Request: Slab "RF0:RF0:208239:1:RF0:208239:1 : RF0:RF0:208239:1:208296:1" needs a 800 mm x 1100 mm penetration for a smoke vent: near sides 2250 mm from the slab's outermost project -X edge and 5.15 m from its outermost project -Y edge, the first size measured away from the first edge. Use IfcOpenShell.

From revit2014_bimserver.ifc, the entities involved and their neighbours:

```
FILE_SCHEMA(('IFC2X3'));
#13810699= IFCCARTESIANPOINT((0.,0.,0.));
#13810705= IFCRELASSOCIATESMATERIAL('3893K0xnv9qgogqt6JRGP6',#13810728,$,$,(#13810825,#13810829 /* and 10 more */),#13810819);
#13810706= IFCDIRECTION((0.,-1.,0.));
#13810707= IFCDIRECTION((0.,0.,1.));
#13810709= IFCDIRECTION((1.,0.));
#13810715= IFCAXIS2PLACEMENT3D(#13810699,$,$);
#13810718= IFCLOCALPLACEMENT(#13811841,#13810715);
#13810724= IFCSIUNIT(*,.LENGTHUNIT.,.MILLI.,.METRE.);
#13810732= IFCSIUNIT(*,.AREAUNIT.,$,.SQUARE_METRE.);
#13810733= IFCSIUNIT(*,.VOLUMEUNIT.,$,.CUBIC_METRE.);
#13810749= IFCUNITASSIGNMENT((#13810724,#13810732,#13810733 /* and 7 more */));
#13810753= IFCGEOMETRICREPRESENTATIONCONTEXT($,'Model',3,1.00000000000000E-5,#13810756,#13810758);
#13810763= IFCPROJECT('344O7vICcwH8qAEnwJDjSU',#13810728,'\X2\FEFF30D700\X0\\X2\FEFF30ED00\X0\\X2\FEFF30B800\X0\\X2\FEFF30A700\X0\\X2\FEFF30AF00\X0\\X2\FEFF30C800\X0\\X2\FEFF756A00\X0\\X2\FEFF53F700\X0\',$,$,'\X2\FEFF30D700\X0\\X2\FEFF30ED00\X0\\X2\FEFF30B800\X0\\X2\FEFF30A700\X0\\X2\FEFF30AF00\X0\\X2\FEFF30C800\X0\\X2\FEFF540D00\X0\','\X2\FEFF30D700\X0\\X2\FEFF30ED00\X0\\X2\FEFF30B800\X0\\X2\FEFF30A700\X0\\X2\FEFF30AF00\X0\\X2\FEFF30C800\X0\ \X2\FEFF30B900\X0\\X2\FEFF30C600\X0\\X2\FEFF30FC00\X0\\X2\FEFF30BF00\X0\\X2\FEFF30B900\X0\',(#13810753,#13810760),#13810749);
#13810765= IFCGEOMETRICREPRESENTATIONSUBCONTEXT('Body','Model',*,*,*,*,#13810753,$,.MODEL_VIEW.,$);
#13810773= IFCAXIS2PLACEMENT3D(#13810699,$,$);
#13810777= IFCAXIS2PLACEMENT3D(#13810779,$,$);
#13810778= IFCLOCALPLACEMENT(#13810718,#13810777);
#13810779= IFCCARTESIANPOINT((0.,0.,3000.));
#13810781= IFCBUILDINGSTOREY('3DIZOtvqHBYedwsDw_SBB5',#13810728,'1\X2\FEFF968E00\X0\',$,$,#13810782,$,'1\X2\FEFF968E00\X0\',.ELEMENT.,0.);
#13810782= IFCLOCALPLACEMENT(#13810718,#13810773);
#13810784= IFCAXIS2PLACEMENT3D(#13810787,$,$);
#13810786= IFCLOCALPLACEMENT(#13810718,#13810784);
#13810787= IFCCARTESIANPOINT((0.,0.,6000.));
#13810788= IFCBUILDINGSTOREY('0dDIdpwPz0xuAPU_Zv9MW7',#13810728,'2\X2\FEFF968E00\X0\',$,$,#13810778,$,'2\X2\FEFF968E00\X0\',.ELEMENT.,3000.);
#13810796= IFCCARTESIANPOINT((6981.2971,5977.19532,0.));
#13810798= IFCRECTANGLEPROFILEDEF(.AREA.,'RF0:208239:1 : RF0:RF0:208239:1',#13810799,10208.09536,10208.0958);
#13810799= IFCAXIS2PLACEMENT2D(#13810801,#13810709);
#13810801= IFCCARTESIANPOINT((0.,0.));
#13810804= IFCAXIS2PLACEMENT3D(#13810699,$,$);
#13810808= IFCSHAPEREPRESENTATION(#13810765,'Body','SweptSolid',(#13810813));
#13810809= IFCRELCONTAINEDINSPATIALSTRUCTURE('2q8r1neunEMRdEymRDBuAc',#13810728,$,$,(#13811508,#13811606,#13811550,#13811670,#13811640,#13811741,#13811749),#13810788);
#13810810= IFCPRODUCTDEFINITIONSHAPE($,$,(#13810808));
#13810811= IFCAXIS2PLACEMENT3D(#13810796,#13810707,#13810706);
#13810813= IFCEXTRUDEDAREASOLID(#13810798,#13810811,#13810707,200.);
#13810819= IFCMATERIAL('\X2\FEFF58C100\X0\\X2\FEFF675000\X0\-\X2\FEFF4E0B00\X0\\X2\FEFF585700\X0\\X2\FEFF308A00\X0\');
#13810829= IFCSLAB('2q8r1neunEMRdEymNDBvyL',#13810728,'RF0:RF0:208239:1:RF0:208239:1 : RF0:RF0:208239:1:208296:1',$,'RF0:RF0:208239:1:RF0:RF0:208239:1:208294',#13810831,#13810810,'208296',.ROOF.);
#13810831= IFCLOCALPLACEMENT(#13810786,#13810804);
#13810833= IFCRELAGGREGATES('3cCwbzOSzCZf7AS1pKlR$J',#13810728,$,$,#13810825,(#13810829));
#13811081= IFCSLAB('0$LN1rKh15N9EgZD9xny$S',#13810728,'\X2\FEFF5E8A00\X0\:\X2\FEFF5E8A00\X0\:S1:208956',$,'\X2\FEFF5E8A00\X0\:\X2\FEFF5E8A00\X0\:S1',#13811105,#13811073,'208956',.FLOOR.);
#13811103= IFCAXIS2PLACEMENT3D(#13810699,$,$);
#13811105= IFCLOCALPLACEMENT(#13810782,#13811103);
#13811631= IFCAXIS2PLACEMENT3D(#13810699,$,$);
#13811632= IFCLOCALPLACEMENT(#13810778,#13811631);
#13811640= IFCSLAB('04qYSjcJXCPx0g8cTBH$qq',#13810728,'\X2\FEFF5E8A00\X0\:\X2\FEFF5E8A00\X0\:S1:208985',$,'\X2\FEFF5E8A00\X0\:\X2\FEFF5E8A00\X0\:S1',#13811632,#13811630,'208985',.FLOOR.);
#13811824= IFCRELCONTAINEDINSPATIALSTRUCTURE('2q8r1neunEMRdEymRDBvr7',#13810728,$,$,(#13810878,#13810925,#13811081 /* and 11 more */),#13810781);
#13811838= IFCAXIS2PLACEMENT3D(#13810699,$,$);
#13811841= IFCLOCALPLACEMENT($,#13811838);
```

```python
import numpy as np
import ifcopenshell
import ifcopenshell.api.feature
import ifcopenshell.api.geometry
import ifcopenshell.api.root
import ifcopenshell.geom
import ifcopenshell.util.placement
import ifcopenshell.util.representation
import ifcopenshell.util.shape
import ifcopenshell.util.unit

model = ifcopenshell.open("revit2014_bimserver.ifc")
unit_scale = ifcopenshell.util.unit.calculate_unit_scale(model)
settings = ifcopenshell.geom.settings()


def volume(element):
    """Net volume in cubic metres, openings subtracted."""
    shape = ifcopenshell.geom.create_shape(settings, element)
    return ifcopenshell.util.shape.get_volume(shape.geometry)


slab = model.by_id(13810829)
before = volume(slab)

# Extent in the slab's own axes, in metres. The edges named are its -X and -Y sides.
slab_shape = ifcopenshell.geom.create_shape(settings, slab)
vertices = ifcopenshell.util.shape.get_vertices(slab_shape.geometry)
x_min, y_min, bottom = vertices.min(axis=0)
top = vertices[:, 2].max()

opening = ifcopenshell.api.root.create_entity(model, ifc_class="IfcOpeningElement", name="Smoke vent opening")
context = ifcopenshell.util.representation.get_context(model, "Model", "Body", "MODEL_VIEW")
width, depth = 0.8, 1.1
outline = [(0.0, 0.0), (width, 0.0), (width, depth), (0.0, depth), (0.0, 0.0)]
# Overshoot both faces by 50 mm so the cut is clean.
shape = ifcopenshell.api.geometry.add_slab_representation(
    model, context=context, depth=top - bottom + 0.1, polyline=outline
)
ifcopenshell.api.geometry.assign_representation(model, product=opening, representation=shape)

matrix = ifcopenshell.util.placement.get_local_placement(slab.ObjectPlacement)
matrix[:, 3] = matrix @ np.append(np.array([x_min + 2.25, y_min + 5.15, bottom - 0.05]) / unit_scale, 1.0)
ifcopenshell.api.geometry.edit_object_placement(model, product=opening, matrix=matrix, is_si=False)
ifcopenshell.api.feature.add_feature(model, feature=opening, element=slab)

after = volume(slab)

print(f"slab volume {before:.3f} -> {after:.3f} m3")

model.write("revit2014_bimserver_v2.ifc")
```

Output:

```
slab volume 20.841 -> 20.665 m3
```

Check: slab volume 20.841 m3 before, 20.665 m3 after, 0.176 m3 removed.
